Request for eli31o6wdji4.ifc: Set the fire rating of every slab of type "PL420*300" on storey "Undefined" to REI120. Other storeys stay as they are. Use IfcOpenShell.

First a look at what the model holds.

```python
import ifcopenshell
import ifcopenshell.util.element

model = ifcopenshell.open("eli31o6wdji4.ifc")
print(model.schema)
storey = next(s for s in model.by_type("IfcBuildingStorey") if s.Name == "Undefined")
slabs = [e for e in ifcopenshell.util.element.get_decomposition(storey) if e.is_a("IfcSlab")]
seen = {}
for e in slabs:
    element_type = ifcopenshell.util.element.get_type(e)
    key = (element_type.Name if element_type != e and element_type else None, ifcopenshell.util.element.get_pset(e, "Pset_SlabCommon", "FireRating"))
    seen[key] = seen.get(key, 0) + 1
for (name, value), count in sorted(seen.items(), key=str):
    print(count, "x", name, "|", value)
```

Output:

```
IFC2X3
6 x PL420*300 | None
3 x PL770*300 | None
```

```python
import ifcopenshell
import ifcopenshell.api.pset
import ifcopenshell.util.element

model = ifcopenshell.open("eli31o6wdji4.ifc")

storey = next(s for s in model.by_type("IfcBuildingStorey") if s.Name == "Undefined")
slabs = [e for e in ifcopenshell.util.element.get_decomposition(storey) if e.is_a("IfcSlab")]

count = 0
for e in slabs:
    element_type = ifcopenshell.util.element.get_type(e)
    if element_type in (None, e) or element_type.Name != "PL420*300":
        continue
    found = ifcopenshell.util.element.get_pset(e, "Pset_SlabCommon", should_inherit=False)
    if found:
        pset = model.by_id(found["id"])
        if len(ifcopenshell.util.element.get_elements_by_pset(pset)) > 1:
            pset = ifcopenshell.api.pset.unshare_pset(model, products=[e], pset=pset)[0]
    else:
        pset = ifcopenshell.api.pset.add_pset(model, product=e, name="Pset_SlabCommon")
    ifcopenshell.api.pset.edit_pset(model, pset=pset, properties={"FireRating": "REI120"})
    count += 1

print(count, "slabs updated")

model.write("eli31o6wdji4_v2.ifc")
```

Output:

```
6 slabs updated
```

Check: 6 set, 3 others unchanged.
